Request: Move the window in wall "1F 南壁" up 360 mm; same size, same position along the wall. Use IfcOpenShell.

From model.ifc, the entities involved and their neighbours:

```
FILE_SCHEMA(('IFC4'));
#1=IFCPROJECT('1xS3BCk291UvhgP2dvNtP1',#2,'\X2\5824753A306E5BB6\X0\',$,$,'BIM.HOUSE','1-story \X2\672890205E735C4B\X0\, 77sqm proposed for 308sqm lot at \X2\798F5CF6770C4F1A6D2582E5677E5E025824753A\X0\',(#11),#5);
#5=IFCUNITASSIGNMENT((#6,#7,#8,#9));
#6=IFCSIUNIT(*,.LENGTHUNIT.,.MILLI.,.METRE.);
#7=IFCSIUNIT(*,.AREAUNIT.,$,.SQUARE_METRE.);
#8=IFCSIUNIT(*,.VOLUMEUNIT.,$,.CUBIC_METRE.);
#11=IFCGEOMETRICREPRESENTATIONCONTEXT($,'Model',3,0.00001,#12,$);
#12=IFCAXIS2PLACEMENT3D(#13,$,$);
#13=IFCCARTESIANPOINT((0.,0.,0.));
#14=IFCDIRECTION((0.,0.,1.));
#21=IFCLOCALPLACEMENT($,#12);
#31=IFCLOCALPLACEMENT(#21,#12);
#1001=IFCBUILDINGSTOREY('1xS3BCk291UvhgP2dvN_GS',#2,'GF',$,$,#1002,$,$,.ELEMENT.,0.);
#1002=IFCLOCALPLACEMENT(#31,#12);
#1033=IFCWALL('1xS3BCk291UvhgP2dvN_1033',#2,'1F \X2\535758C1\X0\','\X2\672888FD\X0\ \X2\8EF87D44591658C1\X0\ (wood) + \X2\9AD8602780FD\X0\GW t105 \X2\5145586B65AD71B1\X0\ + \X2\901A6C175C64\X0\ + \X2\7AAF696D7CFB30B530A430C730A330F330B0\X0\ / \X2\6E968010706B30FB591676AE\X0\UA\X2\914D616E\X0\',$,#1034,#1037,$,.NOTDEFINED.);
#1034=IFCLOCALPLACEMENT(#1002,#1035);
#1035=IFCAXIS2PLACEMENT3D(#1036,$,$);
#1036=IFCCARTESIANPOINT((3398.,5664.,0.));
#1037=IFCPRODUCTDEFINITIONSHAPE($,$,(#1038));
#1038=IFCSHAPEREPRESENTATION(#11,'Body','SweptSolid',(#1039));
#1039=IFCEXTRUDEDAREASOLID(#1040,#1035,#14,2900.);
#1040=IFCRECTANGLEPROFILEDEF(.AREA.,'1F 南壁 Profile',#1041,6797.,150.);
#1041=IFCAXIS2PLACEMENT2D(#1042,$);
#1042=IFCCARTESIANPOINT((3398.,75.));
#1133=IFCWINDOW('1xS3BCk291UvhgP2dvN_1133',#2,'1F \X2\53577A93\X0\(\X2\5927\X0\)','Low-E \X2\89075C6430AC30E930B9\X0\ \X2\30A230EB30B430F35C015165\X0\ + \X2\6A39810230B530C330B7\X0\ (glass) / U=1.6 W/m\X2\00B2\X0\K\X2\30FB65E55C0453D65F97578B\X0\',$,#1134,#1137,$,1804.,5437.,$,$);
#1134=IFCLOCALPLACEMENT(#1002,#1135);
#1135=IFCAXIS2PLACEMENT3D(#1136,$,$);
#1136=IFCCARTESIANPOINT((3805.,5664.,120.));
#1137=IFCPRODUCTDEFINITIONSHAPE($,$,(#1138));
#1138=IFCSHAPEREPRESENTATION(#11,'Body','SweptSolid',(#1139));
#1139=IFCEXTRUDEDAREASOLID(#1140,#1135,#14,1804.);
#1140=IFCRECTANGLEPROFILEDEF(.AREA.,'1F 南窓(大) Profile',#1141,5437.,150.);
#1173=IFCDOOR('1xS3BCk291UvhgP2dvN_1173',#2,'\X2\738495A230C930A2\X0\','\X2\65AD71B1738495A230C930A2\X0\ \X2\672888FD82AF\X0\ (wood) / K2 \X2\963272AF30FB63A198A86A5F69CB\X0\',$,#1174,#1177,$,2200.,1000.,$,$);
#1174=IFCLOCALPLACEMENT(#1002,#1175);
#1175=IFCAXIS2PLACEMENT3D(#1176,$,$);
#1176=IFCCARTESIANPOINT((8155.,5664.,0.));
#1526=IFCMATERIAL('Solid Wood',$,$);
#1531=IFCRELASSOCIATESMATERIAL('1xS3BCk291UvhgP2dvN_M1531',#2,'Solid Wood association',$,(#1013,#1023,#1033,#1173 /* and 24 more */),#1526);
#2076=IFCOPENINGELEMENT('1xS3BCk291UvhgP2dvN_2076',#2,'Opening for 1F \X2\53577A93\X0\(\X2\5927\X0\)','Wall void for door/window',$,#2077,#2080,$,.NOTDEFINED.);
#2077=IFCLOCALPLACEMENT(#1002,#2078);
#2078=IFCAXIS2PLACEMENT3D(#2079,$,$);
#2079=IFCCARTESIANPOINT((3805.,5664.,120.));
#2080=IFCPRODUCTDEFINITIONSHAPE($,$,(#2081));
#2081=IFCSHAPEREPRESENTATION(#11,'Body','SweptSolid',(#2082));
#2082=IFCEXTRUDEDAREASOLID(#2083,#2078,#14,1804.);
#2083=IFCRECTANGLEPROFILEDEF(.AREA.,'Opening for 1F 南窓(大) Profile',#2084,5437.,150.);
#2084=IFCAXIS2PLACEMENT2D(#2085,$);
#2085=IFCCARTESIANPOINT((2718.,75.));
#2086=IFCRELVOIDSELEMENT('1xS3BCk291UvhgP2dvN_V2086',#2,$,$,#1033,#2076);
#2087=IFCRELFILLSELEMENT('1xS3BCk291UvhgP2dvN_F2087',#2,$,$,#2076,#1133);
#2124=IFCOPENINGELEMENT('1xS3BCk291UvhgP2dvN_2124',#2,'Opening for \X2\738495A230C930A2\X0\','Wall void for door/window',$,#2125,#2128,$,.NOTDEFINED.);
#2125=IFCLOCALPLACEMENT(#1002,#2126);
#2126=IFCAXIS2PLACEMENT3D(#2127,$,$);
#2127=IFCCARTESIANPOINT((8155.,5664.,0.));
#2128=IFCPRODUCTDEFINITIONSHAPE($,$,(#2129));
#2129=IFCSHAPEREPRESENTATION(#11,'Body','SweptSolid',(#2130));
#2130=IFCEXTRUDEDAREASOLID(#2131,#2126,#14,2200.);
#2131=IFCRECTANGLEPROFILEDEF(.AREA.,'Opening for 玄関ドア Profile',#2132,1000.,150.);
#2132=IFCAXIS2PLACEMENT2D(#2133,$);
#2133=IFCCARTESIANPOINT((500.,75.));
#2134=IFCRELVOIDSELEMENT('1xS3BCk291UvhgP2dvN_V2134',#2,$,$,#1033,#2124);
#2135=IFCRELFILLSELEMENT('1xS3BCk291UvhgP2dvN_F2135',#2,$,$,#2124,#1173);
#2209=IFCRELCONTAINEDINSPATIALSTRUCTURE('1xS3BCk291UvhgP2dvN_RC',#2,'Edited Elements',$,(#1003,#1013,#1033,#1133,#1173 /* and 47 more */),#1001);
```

```python
import numpy as np
import ifcopenshell
import ifcopenshell.api.geometry
import ifcopenshell.util.placement
import ifcopenshell.util.unit

model = ifcopenshell.open("model.ifc")
unit_scale = ifcopenshell.util.unit.calculate_unit_scale(model)

window = model.by_guid("1xS3BCk291UvhgP2dvN_1133")
opening = window.FillsVoids[0].RelatingOpeningElement
dz = 0.36 / unit_scale

shift = np.array([0.0, 0.0, dz])
# The window is not placed relative to its opening, so move both.
for product in (opening, window):
    matrix = ifcopenshell.util.placement.get_local_placement(product.ObjectPlacement)
    matrix[:3, 3] += shift
    ifcopenshell.api.geometry.edit_object_placement(model, product=product, matrix=matrix, is_si=False)

print(f"moved by {dz * unit_scale:+.3f} m")

model.write("model_rev.ifc")
```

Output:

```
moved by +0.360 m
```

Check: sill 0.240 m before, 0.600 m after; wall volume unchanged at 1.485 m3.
